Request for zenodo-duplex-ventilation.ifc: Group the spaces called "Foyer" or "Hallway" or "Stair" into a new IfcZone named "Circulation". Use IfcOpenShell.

First a look at what the model holds.

```python
import ifcopenshell

model = ifcopenshell.open("zenodo-duplex-ventilation.ifc")
print(model.schema)
seen = {}
for space in model.by_type("IfcSpace"):
    seen[space.LongName] = seen.get(space.LongName, 0) + 1
for name, count in sorted(seen.items(), key=str):
    print(count, "x", name)
print("zones:", [z.Name for z in model.by_type("IfcZone")][:20])
```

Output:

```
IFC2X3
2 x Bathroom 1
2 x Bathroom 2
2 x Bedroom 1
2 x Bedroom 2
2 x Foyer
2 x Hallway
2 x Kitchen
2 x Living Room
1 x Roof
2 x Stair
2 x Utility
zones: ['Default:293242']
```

```python
import ifcopenshell
import ifcopenshell.api.group
import ifcopenshell.api.root

model = ifcopenshell.open("zenodo-duplex-ventilation.ifc")

names = {"Foyer", "Hallway", "Stair"}
spaces = [s for s in model.by_type("IfcSpace") if s.LongName in names]

zone = ifcopenshell.api.root.create_entity(model, ifc_class="IfcZone", name="Circulation")
ifcopenshell.api.group.assign_group(model, products=spaces, group=zone)
print(len(spaces), "spaces in", zone.Name)

model.write("zenodo-duplex-ventilation_edited.ifc")
```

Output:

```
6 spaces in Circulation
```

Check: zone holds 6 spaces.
